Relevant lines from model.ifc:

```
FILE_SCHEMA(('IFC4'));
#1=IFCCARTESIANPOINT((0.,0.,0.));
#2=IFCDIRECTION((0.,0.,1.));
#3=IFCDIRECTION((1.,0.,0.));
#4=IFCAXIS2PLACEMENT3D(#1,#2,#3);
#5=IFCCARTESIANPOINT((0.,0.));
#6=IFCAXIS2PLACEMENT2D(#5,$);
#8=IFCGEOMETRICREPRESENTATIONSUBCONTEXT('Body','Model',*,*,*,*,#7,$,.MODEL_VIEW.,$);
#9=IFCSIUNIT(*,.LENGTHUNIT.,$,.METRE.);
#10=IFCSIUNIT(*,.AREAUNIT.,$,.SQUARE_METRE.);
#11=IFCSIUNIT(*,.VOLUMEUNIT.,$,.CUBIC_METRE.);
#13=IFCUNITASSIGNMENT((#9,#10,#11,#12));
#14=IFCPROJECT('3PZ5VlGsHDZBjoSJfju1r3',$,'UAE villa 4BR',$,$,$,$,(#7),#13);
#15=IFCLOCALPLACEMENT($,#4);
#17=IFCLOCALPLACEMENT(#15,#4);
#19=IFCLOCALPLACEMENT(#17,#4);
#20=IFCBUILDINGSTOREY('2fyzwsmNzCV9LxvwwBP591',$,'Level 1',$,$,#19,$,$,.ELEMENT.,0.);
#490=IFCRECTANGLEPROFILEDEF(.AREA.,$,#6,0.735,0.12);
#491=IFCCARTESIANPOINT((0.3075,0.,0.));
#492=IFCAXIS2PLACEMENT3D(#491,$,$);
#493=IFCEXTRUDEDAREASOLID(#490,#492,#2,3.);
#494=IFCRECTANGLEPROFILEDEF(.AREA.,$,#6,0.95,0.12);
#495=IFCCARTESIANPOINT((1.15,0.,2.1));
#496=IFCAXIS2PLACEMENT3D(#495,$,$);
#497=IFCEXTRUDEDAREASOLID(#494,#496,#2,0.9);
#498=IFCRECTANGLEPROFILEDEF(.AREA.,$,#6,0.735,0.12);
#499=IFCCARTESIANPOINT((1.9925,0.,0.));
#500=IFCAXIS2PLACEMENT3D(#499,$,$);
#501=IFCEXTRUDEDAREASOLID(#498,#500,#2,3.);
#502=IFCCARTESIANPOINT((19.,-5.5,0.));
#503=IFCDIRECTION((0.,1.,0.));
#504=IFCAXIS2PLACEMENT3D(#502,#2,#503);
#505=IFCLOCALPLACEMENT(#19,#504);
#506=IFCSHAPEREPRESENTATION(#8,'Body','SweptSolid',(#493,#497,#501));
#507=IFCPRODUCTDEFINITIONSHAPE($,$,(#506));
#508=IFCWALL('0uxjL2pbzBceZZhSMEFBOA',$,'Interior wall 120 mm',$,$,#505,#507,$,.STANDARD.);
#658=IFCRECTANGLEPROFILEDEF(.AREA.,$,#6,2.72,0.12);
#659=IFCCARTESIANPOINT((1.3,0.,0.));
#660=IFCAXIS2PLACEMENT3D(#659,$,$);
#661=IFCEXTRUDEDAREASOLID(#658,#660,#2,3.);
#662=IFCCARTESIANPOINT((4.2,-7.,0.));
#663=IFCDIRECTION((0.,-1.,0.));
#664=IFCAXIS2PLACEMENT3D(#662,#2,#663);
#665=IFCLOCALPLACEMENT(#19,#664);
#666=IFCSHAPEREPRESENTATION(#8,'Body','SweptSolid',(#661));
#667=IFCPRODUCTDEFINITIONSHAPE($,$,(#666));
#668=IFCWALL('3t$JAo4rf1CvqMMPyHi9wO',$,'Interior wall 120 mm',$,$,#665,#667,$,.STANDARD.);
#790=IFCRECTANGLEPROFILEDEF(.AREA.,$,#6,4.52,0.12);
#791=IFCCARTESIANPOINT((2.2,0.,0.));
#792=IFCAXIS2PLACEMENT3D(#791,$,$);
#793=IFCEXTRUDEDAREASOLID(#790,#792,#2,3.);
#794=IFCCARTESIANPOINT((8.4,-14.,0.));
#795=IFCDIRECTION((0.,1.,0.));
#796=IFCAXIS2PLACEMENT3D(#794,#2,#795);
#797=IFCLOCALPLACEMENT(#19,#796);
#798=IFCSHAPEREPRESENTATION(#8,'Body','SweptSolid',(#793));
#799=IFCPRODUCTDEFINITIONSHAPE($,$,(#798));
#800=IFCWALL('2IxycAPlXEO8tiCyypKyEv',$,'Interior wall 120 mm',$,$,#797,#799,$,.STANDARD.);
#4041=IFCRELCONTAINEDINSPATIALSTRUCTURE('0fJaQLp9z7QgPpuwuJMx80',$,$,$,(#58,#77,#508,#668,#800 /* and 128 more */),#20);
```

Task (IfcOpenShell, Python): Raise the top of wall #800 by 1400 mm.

```python
import ifcopenshell
import ifcopenshell.geom
import ifcopenshell.util.representation
import ifcopenshell.util.shape
import ifcopenshell.util.unit

model = ifcopenshell.open("model.ifc")
unit_scale = ifcopenshell.util.unit.calculate_unit_scale(model)
settings = ifcopenshell.geom.settings()


def volume(element):
    """Net volume in cubic metres, openings subtracted."""
    shape = ifcopenshell.geom.create_shape(settings, element)
    return ifcopenshell.util.shape.get_volume(shape.geometry)


wall = model.by_guid("2IxycAPlXEO8tiCyypKyEv")
before = volume(wall)

body = ifcopenshell.util.representation.get_representation(wall, "Model", "Body")
solid = body.Items[0]
old_height = solid.Depth
solid.Depth += 1.4 / unit_scale
after = volume(wall)

print(f"height {old_height:g} -> {solid.Depth:g}, volume {before:.3f} -> {after:.3f} m3")

model.write("model_rev.ifc")
```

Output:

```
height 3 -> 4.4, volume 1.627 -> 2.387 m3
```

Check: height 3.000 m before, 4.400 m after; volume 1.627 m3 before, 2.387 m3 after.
